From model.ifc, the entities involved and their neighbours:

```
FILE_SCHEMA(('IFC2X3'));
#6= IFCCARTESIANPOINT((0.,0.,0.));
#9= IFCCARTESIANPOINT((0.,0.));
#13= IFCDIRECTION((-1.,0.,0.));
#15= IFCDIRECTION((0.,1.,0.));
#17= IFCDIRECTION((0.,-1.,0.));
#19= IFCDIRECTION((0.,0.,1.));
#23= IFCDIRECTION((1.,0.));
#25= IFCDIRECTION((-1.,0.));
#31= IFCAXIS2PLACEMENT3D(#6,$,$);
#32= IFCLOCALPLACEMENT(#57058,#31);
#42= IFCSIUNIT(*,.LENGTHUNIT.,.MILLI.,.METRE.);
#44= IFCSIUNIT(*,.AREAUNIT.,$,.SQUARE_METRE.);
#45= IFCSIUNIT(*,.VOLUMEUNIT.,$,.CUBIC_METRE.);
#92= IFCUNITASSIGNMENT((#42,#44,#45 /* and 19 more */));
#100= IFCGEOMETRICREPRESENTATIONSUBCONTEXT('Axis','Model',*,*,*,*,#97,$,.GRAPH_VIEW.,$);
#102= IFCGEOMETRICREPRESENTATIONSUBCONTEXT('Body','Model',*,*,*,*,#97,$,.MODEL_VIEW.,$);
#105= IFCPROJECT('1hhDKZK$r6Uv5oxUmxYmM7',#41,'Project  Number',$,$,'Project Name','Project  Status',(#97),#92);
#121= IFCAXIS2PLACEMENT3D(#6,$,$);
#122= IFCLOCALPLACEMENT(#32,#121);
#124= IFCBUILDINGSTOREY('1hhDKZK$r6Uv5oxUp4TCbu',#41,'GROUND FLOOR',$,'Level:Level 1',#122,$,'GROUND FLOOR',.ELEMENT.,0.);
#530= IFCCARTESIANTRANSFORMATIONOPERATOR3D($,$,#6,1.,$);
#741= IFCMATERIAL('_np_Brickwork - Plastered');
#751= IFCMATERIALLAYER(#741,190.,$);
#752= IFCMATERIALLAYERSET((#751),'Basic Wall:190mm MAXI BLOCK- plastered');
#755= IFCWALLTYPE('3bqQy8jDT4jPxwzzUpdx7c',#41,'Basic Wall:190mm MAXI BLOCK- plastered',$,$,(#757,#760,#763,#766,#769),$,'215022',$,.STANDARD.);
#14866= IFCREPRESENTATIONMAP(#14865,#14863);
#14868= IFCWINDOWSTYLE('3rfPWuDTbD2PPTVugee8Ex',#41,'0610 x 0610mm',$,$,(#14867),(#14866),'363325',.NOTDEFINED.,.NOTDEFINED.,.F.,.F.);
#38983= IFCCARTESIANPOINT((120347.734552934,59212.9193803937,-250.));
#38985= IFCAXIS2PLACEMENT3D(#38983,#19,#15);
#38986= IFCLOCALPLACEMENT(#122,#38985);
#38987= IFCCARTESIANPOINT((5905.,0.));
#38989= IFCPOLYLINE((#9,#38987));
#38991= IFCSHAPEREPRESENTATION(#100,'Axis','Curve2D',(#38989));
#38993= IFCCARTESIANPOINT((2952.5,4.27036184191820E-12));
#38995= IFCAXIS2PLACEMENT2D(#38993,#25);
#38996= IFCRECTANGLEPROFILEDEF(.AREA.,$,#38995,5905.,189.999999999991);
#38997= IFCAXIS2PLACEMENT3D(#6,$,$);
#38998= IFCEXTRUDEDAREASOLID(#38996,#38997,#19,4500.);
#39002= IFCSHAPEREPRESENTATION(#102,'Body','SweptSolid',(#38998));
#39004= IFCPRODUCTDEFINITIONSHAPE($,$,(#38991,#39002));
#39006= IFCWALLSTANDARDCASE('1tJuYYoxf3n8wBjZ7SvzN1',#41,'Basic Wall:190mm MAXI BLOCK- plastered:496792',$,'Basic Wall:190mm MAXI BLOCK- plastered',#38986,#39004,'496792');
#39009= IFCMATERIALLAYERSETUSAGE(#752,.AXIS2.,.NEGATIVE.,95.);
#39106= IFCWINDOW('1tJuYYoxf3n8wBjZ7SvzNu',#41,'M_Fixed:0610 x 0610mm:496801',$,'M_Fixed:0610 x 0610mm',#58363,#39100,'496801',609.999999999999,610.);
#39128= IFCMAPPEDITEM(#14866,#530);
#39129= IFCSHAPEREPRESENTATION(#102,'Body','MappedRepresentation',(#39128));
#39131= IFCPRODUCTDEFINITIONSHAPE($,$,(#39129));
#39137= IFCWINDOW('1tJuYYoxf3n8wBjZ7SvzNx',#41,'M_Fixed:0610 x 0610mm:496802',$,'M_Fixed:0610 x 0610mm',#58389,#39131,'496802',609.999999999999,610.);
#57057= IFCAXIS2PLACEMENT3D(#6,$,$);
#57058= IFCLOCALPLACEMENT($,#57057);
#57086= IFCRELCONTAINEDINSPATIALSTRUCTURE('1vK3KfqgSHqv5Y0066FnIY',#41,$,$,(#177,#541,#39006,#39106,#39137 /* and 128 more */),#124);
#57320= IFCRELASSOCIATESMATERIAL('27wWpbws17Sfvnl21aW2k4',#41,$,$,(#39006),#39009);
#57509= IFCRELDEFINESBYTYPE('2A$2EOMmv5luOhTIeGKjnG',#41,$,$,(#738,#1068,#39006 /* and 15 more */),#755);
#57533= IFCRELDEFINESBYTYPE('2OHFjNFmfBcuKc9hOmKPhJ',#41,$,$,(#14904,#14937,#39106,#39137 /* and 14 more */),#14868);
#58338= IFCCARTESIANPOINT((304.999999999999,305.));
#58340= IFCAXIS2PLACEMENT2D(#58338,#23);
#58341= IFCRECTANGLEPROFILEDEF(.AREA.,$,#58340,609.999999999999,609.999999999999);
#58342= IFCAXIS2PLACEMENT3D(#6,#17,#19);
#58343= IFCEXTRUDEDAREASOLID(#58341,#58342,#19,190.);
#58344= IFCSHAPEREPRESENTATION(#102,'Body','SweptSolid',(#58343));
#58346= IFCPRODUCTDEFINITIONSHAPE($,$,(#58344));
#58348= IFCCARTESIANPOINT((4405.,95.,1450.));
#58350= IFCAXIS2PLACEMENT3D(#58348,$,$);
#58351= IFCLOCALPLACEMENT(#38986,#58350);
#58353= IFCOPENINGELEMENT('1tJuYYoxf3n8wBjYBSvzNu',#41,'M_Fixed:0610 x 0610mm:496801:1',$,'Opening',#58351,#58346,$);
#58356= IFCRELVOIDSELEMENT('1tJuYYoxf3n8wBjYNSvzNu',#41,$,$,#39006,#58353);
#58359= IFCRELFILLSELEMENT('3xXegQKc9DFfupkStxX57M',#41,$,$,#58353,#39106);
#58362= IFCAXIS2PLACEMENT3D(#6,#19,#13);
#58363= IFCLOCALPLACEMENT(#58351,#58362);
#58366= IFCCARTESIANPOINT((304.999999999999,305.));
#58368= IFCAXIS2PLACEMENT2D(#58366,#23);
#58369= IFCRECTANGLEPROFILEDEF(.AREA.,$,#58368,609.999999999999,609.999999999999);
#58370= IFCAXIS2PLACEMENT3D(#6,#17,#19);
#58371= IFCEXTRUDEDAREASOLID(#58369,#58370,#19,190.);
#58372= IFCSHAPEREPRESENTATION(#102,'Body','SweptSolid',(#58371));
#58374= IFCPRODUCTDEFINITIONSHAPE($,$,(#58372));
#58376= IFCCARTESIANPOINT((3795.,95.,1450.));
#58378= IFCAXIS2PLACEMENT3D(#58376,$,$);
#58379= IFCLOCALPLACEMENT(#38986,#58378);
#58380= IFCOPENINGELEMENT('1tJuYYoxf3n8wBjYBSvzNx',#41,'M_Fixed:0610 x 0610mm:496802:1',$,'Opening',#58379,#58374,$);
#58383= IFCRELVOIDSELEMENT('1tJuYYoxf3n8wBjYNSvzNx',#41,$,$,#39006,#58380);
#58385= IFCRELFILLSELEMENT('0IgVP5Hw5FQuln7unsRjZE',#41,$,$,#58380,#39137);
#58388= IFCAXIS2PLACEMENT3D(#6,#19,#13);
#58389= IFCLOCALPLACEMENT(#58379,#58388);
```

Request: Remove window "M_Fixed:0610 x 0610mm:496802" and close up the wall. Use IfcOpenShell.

```python
import ifcopenshell
import ifcopenshell.api.feature
import ifcopenshell.api.root
import ifcopenshell.geom
import ifcopenshell.util.shape

model = ifcopenshell.open("model.ifc")
settings = ifcopenshell.geom.settings()


def volume(element):
    """Net volume in cubic metres, openings subtracted."""
    shape = ifcopenshell.geom.create_shape(settings, element)
    return ifcopenshell.util.shape.get_volume(shape.geometry)


window = model.by_guid("1tJuYYoxf3n8wBjZ7SvzNx")
opening = window.FillsVoids[0].RelatingOpeningElement
wall = opening.VoidsElements[0].RelatingBuildingElement
before = volume(wall)

ifcopenshell.api.root.remove_product(model, product=window)
ifcopenshell.api.feature.remove_feature(model, feature=opening)

after = volume(wall)

print(f"wall volume {before:.3f} -> {after:.3f} m3")

model.write("model-out.ifc")
```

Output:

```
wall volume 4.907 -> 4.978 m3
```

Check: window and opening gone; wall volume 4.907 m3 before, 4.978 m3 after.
